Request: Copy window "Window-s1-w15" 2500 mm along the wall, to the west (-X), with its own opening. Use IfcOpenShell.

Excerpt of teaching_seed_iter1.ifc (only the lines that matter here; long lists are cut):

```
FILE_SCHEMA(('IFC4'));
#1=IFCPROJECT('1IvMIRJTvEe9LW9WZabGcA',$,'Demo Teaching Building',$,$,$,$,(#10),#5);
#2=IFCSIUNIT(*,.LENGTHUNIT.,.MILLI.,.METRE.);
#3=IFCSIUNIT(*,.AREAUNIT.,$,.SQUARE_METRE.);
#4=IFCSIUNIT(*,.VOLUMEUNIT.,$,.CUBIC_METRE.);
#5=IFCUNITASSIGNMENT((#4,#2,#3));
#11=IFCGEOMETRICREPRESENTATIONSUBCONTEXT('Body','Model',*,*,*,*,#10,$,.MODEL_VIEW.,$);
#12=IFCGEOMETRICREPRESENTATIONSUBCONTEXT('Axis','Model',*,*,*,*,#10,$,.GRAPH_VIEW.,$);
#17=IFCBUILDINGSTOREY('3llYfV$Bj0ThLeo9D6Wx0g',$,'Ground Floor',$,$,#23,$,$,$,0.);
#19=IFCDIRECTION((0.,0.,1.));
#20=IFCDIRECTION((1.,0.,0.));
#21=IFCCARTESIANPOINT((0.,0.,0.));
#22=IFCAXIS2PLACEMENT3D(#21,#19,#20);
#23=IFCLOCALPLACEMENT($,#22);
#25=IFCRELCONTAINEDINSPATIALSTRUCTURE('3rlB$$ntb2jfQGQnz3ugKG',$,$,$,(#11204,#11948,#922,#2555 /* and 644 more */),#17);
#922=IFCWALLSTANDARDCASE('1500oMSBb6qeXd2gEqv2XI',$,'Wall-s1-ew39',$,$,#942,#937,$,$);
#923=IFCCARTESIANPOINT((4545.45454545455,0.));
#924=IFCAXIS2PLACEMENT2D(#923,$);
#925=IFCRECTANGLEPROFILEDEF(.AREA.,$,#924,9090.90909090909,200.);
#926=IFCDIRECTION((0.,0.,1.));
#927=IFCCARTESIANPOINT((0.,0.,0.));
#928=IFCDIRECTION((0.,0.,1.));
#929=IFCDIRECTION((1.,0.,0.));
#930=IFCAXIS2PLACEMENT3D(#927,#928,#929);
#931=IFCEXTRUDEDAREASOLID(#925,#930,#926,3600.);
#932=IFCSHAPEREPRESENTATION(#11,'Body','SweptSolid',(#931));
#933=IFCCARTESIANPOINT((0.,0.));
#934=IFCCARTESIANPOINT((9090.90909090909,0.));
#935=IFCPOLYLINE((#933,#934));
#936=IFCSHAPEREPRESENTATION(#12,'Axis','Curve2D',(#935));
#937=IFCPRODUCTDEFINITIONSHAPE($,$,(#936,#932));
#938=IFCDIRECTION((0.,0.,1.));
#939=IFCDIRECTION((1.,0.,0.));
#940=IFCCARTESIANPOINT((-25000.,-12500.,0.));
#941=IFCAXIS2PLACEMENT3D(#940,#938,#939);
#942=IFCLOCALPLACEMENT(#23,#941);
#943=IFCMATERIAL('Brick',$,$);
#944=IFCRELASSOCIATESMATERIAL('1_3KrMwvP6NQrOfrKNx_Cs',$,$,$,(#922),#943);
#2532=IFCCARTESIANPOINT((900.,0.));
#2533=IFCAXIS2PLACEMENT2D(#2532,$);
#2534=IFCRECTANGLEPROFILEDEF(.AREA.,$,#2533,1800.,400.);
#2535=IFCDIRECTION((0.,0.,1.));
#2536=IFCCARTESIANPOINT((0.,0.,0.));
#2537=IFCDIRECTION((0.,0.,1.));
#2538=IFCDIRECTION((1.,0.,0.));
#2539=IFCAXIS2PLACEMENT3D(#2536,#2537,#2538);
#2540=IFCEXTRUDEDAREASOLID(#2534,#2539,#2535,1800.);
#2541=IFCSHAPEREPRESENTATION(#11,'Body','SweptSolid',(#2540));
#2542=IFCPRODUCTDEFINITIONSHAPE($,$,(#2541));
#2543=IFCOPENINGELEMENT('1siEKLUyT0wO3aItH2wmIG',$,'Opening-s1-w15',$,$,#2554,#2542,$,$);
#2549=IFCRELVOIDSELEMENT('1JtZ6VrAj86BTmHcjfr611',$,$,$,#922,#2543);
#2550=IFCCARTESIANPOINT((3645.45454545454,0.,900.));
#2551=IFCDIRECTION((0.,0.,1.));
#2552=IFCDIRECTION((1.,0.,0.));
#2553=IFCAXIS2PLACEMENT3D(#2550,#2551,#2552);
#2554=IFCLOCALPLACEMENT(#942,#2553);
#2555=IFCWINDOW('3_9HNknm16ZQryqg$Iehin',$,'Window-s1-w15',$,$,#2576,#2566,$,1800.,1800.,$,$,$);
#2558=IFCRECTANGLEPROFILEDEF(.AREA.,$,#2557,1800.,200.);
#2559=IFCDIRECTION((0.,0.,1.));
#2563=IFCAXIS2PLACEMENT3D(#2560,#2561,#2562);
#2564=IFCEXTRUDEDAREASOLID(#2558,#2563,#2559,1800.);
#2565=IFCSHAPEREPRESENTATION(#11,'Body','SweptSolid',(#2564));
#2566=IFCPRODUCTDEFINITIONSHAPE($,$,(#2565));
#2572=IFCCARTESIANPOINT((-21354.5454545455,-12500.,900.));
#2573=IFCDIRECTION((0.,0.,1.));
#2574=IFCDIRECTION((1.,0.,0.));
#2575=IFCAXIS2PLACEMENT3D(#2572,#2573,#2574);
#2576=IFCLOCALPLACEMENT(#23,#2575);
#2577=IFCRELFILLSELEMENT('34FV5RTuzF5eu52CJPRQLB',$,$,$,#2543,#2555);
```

```python
import ifcopenshell
import ifcopenshell.api.feature
import ifcopenshell.api.geometry
import ifcopenshell.api.root
import ifcopenshell.geom
import ifcopenshell.util.element
import ifcopenshell.util.placement
import ifcopenshell.util.shape
import ifcopenshell.util.unit

model = ifcopenshell.open("teaching_seed_iter1.ifc")
unit_scale = ifcopenshell.util.unit.calculate_unit_scale(model)
settings = ifcopenshell.geom.settings()


def volume(element):
    """Net volume in cubic metres, openings subtracted."""
    shape = ifcopenshell.geom.create_shape(settings, element)
    return ifcopenshell.util.shape.get_volume(shape.geometry)


window = model.by_guid("3_9HNknm16ZQryqg$Iehin")
opening = window.FillsVoids[0].RelatingOpeningElement
wall = opening.VoidsElements[0].RelatingBuildingElement
before = volume(wall)
shift = ifcopenshell.util.placement.get_local_placement(wall.ObjectPlacement)[:3, 0] * -2.5 / unit_scale

# copy_class copies the void relationship, type, container and properties, but no geometry.
new_opening = ifcopenshell.api.root.copy_class(model, product=opening)
new_opening.Representation = ifcopenshell.util.element.copy_deep(
    model, opening.Representation, exclude=["IfcGeometricRepresentationContext", "IfcRepresentationMap"]
)
new_window = ifcopenshell.api.root.copy_class(model, product=window)
new_window.Representation = ifcopenshell.util.element.copy_deep(
    model, window.Representation, exclude=["IfcGeometricRepresentationContext", "IfcRepresentationMap"]
)
ifcopenshell.api.feature.add_filling(model, opening=new_opening, element=new_window)

for old, new in ((opening, new_opening), (window, new_window)):
    matrix = ifcopenshell.util.placement.get_local_placement(old.ObjectPlacement)
    matrix[:3, 3] += shift
    ifcopenshell.api.geometry.edit_object_placement(model, product=new, matrix=matrix, is_si=False)

after = volume(wall)

print(f"wall volume {before:.3f} -> {after:.3f} m3")

model.write("teaching_seed_iter1_v2.ifc")
```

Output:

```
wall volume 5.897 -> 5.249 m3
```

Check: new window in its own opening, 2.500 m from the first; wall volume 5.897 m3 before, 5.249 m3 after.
